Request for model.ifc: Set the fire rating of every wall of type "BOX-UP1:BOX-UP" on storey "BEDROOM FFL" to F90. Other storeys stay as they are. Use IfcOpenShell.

First a look at what the model holds.

```python
import ifcopenshell
import ifcopenshell.util.element

model = ifcopenshell.open("model.ifc")
print(model.schema)
storey = next(s for s in model.by_type("IfcBuildingStorey") if s.Name == "BEDROOM FFL")
walls = [e for e in ifcopenshell.util.element.get_decomposition(storey) if e.is_a("IfcWall")]
seen = {}
for e in walls:
    element_type = ifcopenshell.util.element.get_type(e)
    key = (element_type.Name if element_type != e and element_type else None, ifcopenshell.util.element.get_pset(e, "Pset_WallCommon", "FireRating"))
    seen[key] = seen.get(key, 0) + 1
for (name, value), count in sorted(seen.items(), key=str):
    print(count, "x", name, "|", value)
```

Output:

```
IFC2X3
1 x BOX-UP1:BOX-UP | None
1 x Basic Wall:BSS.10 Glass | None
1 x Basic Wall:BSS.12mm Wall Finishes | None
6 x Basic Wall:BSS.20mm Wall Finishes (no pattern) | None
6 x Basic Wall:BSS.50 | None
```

```python
import ifcopenshell
import ifcopenshell.api.pset
import ifcopenshell.util.element

model = ifcopenshell.open("model.ifc")

storey = next(s for s in model.by_type("IfcBuildingStorey") if s.Name == "BEDROOM FFL")
walls = [e for e in ifcopenshell.util.element.get_decomposition(storey) if e.is_a("IfcWall")]

count = 0
for e in walls:
    element_type = ifcopenshell.util.element.get_type(e)
    if element_type in (None, e) or element_type.Name != "BOX-UP1:BOX-UP":
        continue
    # add_pset returns the element's existing set when there is one.
    pset = ifcopenshell.api.pset.add_pset(model, product=e, name="Pset_WallCommon")
    ifcopenshell.api.pset.edit_pset(model, pset=pset, properties={"FireRating": "F90"})
    count += 1

print(count, "walls updated")

model.write("model_rev.ifc")
```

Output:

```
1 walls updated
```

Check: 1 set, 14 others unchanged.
